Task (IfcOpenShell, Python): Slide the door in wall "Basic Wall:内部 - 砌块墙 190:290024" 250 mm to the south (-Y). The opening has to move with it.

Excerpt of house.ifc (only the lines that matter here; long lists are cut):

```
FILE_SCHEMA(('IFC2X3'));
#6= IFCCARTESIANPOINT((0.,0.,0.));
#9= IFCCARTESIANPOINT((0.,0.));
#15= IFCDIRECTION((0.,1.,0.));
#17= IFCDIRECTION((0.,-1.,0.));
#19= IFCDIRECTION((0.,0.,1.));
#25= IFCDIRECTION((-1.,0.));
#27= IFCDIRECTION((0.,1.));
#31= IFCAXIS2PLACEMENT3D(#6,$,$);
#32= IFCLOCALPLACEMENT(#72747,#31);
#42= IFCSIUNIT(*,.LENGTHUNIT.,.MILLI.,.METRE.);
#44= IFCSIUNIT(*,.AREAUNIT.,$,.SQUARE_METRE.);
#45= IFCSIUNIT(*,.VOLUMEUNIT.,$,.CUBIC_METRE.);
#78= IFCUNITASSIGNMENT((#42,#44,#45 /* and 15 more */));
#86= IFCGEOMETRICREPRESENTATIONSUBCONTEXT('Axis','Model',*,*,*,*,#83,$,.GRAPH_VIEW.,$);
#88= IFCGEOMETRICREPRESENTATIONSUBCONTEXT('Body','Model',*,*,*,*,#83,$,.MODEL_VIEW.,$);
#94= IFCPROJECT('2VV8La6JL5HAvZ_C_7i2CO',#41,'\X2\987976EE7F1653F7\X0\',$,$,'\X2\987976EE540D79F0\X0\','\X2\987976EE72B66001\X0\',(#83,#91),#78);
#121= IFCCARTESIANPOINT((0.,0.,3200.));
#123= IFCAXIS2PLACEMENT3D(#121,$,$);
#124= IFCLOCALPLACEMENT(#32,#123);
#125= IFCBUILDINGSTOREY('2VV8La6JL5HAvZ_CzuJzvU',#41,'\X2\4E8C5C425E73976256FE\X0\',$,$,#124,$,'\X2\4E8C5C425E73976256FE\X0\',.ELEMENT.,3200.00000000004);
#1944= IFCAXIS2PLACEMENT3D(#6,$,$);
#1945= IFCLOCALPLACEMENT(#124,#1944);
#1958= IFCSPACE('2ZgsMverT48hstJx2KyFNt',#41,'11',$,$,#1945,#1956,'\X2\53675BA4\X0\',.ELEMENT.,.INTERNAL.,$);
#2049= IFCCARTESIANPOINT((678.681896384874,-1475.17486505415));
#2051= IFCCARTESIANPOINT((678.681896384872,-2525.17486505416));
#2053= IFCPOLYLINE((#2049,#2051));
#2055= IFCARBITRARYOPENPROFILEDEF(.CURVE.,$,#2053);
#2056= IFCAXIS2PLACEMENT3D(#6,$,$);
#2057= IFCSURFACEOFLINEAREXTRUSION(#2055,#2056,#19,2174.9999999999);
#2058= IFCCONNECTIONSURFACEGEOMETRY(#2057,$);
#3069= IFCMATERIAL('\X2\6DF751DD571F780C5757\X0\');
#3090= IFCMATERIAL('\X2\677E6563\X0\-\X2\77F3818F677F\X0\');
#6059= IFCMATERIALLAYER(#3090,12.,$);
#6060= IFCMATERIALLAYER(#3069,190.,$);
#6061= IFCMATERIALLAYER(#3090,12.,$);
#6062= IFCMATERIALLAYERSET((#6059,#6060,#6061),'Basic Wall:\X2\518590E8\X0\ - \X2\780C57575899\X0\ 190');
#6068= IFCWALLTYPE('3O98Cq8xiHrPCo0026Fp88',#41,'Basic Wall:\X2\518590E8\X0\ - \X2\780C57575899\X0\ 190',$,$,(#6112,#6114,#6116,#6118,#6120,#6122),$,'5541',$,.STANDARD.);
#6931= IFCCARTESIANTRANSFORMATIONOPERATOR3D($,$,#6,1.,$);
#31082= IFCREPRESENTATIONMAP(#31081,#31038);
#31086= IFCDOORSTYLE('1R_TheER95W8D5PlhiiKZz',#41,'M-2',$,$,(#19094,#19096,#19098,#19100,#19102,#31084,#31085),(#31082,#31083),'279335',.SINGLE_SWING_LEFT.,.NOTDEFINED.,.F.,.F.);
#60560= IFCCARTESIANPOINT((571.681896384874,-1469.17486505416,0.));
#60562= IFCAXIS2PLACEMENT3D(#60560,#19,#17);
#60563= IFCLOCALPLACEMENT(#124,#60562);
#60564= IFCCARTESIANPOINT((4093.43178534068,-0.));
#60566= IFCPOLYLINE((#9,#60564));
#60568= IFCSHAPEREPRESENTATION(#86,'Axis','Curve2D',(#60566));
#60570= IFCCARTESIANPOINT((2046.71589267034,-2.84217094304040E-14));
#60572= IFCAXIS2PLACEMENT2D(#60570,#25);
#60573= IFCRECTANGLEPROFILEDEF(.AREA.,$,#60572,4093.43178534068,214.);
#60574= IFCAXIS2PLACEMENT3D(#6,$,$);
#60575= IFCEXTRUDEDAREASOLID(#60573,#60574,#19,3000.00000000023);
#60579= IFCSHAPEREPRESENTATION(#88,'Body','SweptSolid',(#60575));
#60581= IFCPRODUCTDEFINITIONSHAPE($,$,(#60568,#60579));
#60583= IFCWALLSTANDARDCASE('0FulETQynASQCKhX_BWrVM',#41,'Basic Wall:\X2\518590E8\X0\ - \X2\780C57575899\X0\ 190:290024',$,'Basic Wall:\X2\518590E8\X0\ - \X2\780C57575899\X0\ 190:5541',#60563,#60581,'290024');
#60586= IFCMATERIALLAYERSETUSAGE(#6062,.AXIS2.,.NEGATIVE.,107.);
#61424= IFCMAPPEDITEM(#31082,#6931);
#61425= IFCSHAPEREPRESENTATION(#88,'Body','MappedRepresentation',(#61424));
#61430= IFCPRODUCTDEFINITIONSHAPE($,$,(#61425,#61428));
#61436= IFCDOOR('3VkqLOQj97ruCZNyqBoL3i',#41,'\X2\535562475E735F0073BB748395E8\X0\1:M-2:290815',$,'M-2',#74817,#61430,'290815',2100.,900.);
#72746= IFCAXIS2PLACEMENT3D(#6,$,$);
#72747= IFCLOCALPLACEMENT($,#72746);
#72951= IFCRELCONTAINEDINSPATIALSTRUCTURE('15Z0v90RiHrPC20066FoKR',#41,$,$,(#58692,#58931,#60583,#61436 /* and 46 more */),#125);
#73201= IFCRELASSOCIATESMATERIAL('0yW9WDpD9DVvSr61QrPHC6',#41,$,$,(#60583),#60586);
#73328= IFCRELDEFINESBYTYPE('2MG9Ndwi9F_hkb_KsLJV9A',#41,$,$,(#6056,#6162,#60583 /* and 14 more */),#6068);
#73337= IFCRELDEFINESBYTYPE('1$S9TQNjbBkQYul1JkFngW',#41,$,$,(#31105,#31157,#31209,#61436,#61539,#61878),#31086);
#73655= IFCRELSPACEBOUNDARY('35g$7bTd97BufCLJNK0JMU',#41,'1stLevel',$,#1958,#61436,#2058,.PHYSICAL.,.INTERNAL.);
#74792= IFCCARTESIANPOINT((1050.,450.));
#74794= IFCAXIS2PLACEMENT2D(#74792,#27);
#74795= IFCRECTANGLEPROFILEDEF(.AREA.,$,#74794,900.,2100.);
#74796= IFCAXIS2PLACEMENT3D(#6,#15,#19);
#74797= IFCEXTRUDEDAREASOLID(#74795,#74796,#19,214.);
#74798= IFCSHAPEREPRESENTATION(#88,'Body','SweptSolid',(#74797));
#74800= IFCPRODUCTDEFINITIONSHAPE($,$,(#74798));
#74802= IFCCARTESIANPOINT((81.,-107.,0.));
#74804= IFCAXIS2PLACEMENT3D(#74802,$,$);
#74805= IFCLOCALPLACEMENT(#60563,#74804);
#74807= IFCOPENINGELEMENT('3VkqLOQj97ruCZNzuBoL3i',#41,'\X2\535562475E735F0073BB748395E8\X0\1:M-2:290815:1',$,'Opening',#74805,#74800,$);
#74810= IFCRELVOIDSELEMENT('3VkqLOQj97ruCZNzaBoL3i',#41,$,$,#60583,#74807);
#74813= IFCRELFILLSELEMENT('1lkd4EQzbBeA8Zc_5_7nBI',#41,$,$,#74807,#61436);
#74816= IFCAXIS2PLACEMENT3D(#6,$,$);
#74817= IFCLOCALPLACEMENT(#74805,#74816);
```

```python
import numpy as np
import ifcopenshell
import ifcopenshell.api.geometry
import ifcopenshell.util.placement
import ifcopenshell.util.unit

model = ifcopenshell.open("house.ifc")
unit_scale = ifcopenshell.util.unit.calculate_unit_scale(model)

door = model.by_guid("3VkqLOQj97ruCZNyqBoL3i")
opening = door.FillsVoids[0].RelatingOpeningElement
wall = opening.VoidsElements[0].RelatingBuildingElement

wall_matrix = ifcopenshell.util.placement.get_local_placement(wall.ObjectPlacement)
shift = wall_matrix[:3, 0] * 0.25 / unit_scale
before = ifcopenshell.util.placement.get_local_placement(door.ObjectPlacement)[:3, 3].copy()

# The door is placed relative to its opening, so it follows when the opening moves.
matrix = ifcopenshell.util.placement.get_local_placement(opening.ObjectPlacement)
matrix[:3, 3] += shift
ifcopenshell.api.geometry.edit_object_placement(
    model, product=opening, matrix=matrix, is_si=False, should_transform_children=True
)

# Space boundary surfaces are stored in each space's coordinates; move them too.
for rel in door.ProvidesBoundaries:
    if not rel.ConnectionGeometry:
        continue
    surface = rel.ConnectionGeometry.SurfaceOnRelatingElement
    space_matrix = ifcopenshell.util.placement.get_local_placement(rel.RelatingSpace.ObjectPlacement)
    point = np.array(surface.Position.Location.Coordinates) + space_matrix[:3, :3].T @ shift
    surface.Position = model.createIfcAxis2Placement3D(
        model.createIfcCartesianPoint(point.tolist()), surface.Position.Axis, surface.Position.RefDirection
    )

after = ifcopenshell.util.placement.get_local_placement(door.ObjectPlacement)[:3, 3]
print("door moved by", (after - before).round(3) + 0.0)

model.write("house_v2.ifc")
```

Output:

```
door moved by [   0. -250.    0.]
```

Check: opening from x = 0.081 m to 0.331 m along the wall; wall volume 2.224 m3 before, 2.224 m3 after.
